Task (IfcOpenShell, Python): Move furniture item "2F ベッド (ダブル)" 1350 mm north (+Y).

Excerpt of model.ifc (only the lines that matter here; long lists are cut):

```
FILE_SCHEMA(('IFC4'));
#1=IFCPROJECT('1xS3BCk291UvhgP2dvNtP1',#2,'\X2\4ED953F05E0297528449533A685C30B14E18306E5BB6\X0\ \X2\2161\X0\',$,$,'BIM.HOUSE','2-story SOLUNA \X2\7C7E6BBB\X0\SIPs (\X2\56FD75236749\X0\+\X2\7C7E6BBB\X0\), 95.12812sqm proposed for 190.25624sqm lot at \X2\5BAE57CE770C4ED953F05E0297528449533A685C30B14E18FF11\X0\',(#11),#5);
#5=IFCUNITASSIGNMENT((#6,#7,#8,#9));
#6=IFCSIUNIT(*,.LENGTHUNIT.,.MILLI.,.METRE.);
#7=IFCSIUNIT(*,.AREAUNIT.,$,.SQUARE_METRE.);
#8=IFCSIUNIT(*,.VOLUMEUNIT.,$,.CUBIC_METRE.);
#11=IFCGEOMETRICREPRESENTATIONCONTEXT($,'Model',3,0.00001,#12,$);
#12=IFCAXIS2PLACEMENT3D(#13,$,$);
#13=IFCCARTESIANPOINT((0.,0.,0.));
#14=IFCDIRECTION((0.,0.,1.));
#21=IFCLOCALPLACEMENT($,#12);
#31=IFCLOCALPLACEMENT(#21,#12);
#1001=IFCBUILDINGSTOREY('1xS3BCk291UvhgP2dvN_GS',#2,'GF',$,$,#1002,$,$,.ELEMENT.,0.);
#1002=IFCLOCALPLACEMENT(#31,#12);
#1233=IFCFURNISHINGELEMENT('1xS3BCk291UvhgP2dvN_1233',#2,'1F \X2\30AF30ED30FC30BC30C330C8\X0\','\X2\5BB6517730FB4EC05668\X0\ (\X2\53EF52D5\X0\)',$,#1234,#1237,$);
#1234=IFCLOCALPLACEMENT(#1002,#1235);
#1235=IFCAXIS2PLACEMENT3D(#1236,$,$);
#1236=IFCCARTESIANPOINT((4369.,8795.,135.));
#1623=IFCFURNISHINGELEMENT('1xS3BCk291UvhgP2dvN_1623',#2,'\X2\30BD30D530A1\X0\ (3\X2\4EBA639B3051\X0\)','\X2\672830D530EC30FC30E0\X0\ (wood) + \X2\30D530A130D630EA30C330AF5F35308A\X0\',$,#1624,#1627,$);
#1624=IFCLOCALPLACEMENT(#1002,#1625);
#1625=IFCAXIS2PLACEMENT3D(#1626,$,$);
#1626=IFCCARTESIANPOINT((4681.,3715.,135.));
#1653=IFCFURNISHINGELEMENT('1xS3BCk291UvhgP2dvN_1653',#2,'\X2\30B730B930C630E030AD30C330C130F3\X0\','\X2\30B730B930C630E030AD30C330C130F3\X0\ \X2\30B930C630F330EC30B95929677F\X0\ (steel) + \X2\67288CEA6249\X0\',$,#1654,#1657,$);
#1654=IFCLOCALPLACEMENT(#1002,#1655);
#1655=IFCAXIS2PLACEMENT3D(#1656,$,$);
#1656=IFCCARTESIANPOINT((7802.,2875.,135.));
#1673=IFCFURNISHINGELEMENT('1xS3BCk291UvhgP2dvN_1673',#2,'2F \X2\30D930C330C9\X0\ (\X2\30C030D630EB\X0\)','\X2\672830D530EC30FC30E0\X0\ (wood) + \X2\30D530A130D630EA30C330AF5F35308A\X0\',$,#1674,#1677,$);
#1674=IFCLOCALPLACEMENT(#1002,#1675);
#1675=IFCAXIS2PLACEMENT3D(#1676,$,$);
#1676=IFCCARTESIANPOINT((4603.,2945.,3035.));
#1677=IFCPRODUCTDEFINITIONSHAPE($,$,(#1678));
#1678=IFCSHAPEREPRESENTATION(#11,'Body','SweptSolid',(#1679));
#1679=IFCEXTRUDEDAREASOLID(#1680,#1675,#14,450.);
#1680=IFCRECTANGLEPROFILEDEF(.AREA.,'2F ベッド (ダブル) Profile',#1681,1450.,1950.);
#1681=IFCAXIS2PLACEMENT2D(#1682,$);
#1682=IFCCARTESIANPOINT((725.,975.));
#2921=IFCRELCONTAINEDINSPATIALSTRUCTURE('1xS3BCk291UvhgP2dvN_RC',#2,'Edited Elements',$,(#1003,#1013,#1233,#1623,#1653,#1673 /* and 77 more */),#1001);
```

```python
import ifcopenshell
import ifcopenshell.api.geometry
import ifcopenshell.util.placement
import ifcopenshell.util.unit

model = ifcopenshell.open("model.ifc")
unit_scale = ifcopenshell.util.unit.calculate_unit_scale(model)

item = model.by_guid("1xS3BCk291UvhgP2dvN_1673")
matrix = ifcopenshell.util.placement.get_local_placement(item.ObjectPlacement)
matrix[1, 3] += 1.35 / unit_scale
ifcopenshell.api.geometry.edit_object_placement(model, product=item, matrix=matrix, is_si=False)

print(ifcopenshell.util.placement.get_local_placement(item.ObjectPlacement).round(3) + 0.0)

model.write("model_v2.ifc")
```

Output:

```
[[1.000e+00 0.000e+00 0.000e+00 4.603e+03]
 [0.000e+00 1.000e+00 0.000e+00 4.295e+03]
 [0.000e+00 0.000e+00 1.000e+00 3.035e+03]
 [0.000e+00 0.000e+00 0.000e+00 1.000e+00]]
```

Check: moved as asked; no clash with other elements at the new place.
